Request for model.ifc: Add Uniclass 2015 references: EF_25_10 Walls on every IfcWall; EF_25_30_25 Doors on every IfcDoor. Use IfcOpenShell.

First a look at what the model holds.

```python
import ifcopenshell

model = ifcopenshell.open("model.ifc")
print(model.schema)
print("classifications:", [c.Name for c in model.by_type("IfcClassification")])
for ifc_class in ("IfcDoor", "IfcRoof", "IfcStair", "IfcWall", "IfcWindow"):
    print(ifc_class, len(model.by_type(ifc_class)))
```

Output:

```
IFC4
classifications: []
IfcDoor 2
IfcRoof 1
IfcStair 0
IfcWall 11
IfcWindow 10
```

```python
import ifcopenshell
import ifcopenshell.api.classification

model = ifcopenshell.open("model.ifc")

system = ifcopenshell.api.classification.add_classification(model, classification="Uniclass 2015")

codes = {
    "IfcWall": ("EF_25_10", "Walls"),
    "IfcDoor": ("EF_25_30_25", "Doors"),
}
for ifc_class, (code, name) in codes.items():
    products = model.by_type(ifc_class)
    ifcopenshell.api.classification.add_reference(
        model, products=products, classification=system, identification=code, name=name
    )
    print(code, len(products))

model.write("model-out.ifc")
```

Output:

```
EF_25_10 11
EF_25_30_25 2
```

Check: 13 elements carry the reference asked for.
